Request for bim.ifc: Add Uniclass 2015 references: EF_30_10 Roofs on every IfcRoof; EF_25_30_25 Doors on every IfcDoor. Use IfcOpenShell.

First a look at what the model holds.

```python
import ifcopenshell

model = ifcopenshell.open("bim.ifc")
print(model.schema)
print("classifications:", [c.Name for c in model.by_type("IfcClassification")])
for ifc_class in ("IfcDoor", "IfcRoof", "IfcStair", "IfcWall", "IfcWindow"):
    print(ifc_class, len(model.by_type(ifc_class)))
```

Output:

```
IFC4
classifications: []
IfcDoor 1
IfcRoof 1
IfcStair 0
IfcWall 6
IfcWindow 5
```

```python
import ifcopenshell
import ifcopenshell.api.classification

model = ifcopenshell.open("bim.ifc")

system = ifcopenshell.api.classification.add_classification(model, classification="Uniclass 2015")

codes = {
    "IfcRoof": ("EF_30_10", "Roofs"),
    "IfcDoor": ("EF_25_30_25", "Doors"),
}
for ifc_class, (code, name) in codes.items():
    products = model.by_type(ifc_class)
    ifcopenshell.api.classification.add_reference(
        model, products=products, classification=system, identification=code, name=name
    )
    print(code, len(products))

model.write("bim_edited.ifc")
```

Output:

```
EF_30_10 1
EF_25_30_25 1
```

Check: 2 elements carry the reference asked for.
